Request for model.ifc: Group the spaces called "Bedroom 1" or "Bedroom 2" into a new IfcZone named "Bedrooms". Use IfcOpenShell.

First a look at what the model holds.

```python
import ifcopenshell

model = ifcopenshell.open("model.ifc")
print(model.schema)
seen = {}
for space in model.by_type("IfcSpace"):
    seen[space.LongName] = seen.get(space.LongName, 0) + 1
for name, count in sorted(seen.items(), key=str):
    print(count, "x", name)
print("zones:", [z.Name for z in model.by_type("IfcZone")][:20])
```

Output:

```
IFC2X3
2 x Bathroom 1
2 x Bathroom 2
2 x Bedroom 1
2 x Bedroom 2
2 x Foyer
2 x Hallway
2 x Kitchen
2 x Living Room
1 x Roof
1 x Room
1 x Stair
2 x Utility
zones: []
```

```python
import ifcopenshell
import ifcopenshell.api.group
import ifcopenshell.api.root

model = ifcopenshell.open("model.ifc")

names = {"Bedroom 1", "Bedroom 2"}
spaces = [s for s in model.by_type("IfcSpace") if s.LongName in names]

zone = ifcopenshell.api.root.create_entity(model, ifc_class="IfcZone", name="Bedrooms")
ifcopenshell.api.group.assign_group(model, products=spaces, group=zone)
print(len(spaces), "spaces in", zone.Name)

model.write("model-out.ifc")
```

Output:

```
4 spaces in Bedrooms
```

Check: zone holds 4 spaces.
